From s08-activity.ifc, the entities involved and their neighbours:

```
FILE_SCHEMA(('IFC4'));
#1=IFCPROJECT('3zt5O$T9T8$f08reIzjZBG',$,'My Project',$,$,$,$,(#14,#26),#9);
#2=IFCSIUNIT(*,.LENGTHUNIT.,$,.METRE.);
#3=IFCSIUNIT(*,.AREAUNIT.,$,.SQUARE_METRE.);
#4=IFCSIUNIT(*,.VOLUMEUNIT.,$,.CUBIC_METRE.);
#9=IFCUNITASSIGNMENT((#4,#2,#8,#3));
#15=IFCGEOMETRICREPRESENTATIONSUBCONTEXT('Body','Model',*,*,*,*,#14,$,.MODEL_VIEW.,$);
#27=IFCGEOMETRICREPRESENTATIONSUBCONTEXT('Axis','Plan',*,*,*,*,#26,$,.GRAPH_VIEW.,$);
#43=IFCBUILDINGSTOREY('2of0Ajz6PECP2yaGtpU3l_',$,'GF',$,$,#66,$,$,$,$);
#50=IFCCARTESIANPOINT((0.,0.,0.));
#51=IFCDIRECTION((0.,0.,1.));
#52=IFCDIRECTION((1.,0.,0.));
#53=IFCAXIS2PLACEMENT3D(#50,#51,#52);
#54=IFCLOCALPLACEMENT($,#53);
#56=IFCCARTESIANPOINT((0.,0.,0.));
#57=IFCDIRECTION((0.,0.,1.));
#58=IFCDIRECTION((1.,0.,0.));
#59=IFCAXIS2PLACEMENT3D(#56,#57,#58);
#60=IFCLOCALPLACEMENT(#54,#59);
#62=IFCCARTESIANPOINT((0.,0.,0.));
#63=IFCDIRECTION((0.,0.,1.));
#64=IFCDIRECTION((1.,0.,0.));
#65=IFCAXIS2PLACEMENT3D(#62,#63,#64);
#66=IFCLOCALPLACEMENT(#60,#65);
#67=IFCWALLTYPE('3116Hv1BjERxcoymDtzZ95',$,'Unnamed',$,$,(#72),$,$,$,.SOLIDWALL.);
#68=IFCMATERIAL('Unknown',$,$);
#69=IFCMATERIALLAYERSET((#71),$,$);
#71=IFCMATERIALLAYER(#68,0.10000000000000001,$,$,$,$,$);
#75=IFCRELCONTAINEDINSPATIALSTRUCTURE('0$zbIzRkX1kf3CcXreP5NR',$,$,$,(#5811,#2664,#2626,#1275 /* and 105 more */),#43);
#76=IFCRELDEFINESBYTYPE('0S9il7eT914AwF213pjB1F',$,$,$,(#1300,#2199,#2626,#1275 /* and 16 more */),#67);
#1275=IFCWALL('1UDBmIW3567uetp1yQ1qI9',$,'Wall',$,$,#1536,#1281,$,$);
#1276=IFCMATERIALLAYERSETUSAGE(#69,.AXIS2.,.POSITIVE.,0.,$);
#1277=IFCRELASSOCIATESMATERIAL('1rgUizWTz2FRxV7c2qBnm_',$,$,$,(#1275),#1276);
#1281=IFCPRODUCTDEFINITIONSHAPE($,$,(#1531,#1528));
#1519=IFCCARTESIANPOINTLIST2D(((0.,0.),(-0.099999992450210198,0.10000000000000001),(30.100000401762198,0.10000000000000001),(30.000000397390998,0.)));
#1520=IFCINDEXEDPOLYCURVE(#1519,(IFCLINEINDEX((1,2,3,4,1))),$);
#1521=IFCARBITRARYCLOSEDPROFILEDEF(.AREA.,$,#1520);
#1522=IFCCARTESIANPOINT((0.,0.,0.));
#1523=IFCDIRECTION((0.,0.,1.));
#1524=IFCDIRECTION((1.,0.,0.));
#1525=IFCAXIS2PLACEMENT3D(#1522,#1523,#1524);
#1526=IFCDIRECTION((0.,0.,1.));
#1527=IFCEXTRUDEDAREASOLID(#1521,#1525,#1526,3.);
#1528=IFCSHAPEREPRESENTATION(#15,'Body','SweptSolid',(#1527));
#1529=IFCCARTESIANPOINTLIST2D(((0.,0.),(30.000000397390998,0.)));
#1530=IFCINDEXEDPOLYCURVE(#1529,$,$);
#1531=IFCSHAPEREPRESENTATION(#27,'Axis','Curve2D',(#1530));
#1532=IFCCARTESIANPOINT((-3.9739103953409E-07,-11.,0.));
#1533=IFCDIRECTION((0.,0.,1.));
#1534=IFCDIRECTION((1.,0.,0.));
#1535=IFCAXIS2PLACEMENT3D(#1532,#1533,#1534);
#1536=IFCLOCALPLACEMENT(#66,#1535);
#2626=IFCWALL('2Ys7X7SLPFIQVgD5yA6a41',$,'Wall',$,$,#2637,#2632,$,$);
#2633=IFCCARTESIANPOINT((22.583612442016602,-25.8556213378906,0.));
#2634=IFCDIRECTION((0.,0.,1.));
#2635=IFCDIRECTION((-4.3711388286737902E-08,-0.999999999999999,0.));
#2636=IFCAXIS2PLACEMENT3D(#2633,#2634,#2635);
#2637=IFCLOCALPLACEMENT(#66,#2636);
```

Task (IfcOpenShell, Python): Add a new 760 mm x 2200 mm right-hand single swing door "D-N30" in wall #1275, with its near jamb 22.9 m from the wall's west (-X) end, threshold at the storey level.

```python
import numpy as np
import ifcopenshell
import ifcopenshell.api.feature
import ifcopenshell.api.geometry
import ifcopenshell.api.root
import ifcopenshell.api.spatial
import ifcopenshell.geom
import ifcopenshell.util.element
import ifcopenshell.util.placement
import ifcopenshell.util.representation
import ifcopenshell.util.shape
import ifcopenshell.util.unit

model = ifcopenshell.open("s08-activity.ifc")
unit_scale = ifcopenshell.util.unit.calculate_unit_scale(model)
settings = ifcopenshell.geom.settings()


def volume(element):
    """Net volume in cubic metres, openings subtracted."""
    shape = ifcopenshell.geom.create_shape(settings, element)
    return ifcopenshell.util.shape.get_volume(shape.geometry)


wall = model.by_id(1275)
storey = ifcopenshell.util.element.get_container(wall, ifc_class="IfcBuildingStorey")
context = ifcopenshell.util.representation.get_context(model, "Model", "Body", "MODEL_VIEW")
before = volume(wall)

width, height, from_end, sill = 0.76, 2.2, 22.9, 0.0  # metres

# The wall runs along its own X axis, and the end named is its -X end.
wall_shape = ifcopenshell.geom.create_shape(settings, wall)
x, y, z = ifcopenshell.util.shape.get_vertices(wall_shape.geometry).T
start = x.min() + from_end
face, thickness = float(y.min()), float(y.max() - y.min())
wall_matrix = ifcopenshell.util.placement.get_local_placement(wall.ObjectPlacement)
level = ifcopenshell.util.placement.get_local_placement(storey.ObjectPlacement)[2, 3]


def in_wall(x, y):
    """Placement at x, y metres in the wall's axes, at sill height."""
    matrix = wall_matrix.copy()
    matrix[:, 3] = wall_matrix @ np.array([x / unit_scale, y / unit_scale, 0.0, 1.0])
    matrix[2, 3] = level + sill / unit_scale
    return matrix


# Opening: a box that overshoots both wall faces by 50 mm.
opening = ifcopenshell.api.root.create_entity(model, ifc_class="IfcOpeningElement", predefined_type="OPENING")
box = ifcopenshell.api.geometry.add_wall_representation(
    model, context=context, length=width, height=height, thickness=thickness + 0.1
)
ifcopenshell.api.geometry.assign_representation(model, product=opening, representation=box)
ifcopenshell.api.geometry.edit_object_placement(model, product=opening, matrix=in_wall(start, face - 0.05), is_si=False)
ifcopenshell.api.feature.add_feature(model, feature=opening, element=wall)

door = ifcopenshell.api.root.create_entity(model, ifc_class="IfcDoor", name="D-N30", predefined_type="DOOR")
door.OverallWidth, door.OverallHeight = width / unit_scale, height / unit_scale
door.OperationType = "SINGLE_SWING_RIGHT"
body = ifcopenshell.api.geometry.add_door_representation(
    model,
    context=context,
    overall_width=door.OverallWidth,
    overall_height=door.OverallHeight,
    operation_type="SINGLE_SWING_RIGHT",
    lining_properties={"LiningDepth": thickness / unit_scale, "ThresholdDepth": thickness / unit_scale},
)
ifcopenshell.api.geometry.assign_representation(model, product=door, representation=body)
ifcopenshell.api.spatial.assign_container(model, products=[door], relating_structure=storey)
ifcopenshell.api.feature.add_filling(model, opening=opening, element=door)

# The lining spans the wall, so the door starts at the wall face.
ifcopenshell.api.geometry.edit_object_placement(model, product=door, matrix=in_wall(start, face), is_si=False)

after = volume(wall)

print(f"wall volume {before:.3f} -> {after:.3f} m3")

model.write("s08-activity_updated.ifc")
```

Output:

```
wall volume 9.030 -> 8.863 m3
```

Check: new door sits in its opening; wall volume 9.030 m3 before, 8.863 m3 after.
